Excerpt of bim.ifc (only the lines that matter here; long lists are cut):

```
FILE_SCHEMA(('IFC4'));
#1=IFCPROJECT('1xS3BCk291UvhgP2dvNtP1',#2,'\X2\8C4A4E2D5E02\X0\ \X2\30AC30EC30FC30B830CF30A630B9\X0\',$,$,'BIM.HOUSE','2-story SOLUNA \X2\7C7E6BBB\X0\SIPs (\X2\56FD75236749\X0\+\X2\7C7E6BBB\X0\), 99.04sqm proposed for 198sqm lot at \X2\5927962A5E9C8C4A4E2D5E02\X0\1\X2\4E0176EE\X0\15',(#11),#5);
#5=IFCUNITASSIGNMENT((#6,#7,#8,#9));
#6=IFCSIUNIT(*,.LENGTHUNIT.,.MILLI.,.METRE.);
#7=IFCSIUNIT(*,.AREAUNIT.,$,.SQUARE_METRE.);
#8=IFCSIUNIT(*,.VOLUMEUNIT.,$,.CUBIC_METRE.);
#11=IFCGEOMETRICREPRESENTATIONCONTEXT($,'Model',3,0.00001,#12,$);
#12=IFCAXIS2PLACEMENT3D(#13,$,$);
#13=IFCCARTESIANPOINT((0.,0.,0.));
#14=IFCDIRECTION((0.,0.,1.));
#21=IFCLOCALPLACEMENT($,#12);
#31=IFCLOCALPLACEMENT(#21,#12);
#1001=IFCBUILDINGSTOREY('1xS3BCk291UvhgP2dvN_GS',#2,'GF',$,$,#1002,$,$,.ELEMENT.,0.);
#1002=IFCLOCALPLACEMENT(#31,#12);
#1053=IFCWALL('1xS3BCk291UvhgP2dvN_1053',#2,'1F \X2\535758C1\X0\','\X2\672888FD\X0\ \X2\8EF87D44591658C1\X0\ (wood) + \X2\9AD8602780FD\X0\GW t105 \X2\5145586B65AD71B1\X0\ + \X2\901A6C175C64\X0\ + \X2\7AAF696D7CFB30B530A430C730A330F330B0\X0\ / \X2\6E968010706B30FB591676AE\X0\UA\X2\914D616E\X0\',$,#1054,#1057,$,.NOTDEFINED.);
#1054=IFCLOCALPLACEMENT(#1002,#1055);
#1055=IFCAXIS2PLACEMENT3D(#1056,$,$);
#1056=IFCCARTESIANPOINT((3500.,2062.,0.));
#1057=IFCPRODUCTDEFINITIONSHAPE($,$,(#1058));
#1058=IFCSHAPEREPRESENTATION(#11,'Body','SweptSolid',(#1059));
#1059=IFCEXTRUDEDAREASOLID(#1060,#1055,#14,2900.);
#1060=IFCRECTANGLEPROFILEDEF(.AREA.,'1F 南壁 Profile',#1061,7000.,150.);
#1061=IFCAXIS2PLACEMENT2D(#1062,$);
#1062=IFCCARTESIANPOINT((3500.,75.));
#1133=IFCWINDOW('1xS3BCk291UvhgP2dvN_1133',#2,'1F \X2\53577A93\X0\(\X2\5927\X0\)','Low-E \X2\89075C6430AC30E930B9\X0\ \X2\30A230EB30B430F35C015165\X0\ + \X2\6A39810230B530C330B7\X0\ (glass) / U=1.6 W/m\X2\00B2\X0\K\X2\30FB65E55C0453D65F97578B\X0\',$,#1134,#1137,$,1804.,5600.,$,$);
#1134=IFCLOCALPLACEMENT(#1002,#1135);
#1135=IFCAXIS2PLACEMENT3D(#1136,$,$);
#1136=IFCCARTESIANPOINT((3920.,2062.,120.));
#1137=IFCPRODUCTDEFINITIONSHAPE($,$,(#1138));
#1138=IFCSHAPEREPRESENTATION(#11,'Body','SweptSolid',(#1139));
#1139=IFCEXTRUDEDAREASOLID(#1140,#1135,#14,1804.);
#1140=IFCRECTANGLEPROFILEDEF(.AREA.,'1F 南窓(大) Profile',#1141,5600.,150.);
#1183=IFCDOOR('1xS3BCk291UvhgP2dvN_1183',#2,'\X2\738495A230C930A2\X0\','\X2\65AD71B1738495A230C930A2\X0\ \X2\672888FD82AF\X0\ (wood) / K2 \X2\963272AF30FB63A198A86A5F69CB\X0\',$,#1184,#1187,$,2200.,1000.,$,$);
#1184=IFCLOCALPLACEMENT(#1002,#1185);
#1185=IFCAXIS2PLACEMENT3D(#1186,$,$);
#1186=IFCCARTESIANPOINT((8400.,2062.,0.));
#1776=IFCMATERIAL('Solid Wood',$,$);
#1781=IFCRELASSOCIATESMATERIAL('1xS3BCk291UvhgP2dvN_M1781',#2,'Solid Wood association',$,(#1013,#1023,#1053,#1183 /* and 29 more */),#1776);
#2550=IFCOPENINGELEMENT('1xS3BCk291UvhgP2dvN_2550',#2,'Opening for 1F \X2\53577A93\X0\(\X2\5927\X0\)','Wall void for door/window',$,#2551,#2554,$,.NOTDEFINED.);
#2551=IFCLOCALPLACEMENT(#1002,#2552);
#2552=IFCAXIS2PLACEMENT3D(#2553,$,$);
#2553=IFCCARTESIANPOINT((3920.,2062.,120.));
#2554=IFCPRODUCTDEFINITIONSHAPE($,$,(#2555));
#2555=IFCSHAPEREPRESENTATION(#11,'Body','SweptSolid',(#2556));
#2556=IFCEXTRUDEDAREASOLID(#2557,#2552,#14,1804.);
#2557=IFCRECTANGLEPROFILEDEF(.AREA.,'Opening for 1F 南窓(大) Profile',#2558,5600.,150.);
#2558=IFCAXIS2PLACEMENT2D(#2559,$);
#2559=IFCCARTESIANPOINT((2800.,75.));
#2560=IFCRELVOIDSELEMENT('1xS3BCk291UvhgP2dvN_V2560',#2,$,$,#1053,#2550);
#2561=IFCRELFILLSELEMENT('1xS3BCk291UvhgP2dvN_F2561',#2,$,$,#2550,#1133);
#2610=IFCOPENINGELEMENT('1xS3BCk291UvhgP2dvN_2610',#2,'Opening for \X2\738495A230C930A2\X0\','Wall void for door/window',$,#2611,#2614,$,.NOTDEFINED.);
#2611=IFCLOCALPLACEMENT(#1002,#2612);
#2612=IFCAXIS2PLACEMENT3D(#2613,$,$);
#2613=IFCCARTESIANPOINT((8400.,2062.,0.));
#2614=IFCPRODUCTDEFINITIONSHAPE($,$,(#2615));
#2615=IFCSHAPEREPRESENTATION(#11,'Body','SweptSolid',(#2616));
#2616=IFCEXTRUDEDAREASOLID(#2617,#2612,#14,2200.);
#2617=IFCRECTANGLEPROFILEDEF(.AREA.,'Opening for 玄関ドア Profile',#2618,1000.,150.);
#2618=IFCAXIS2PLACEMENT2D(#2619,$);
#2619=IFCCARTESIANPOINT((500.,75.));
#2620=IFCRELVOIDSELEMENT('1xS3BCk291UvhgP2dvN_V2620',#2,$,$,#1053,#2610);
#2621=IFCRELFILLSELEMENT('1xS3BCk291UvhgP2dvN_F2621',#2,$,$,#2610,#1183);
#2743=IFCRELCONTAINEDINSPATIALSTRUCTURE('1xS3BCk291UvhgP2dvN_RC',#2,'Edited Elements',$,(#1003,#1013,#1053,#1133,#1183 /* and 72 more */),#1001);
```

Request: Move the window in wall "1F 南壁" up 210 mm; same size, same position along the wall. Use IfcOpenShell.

```python
import numpy as np
import ifcopenshell
import ifcopenshell.api.geometry
import ifcopenshell.util.placement
import ifcopenshell.util.unit

model = ifcopenshell.open("bim.ifc")
unit_scale = ifcopenshell.util.unit.calculate_unit_scale(model)

window = model.by_guid("1xS3BCk291UvhgP2dvN_1133")
opening = window.FillsVoids[0].RelatingOpeningElement
dz = 0.21 / unit_scale

shift = np.array([0.0, 0.0, dz])
# The window is not placed relative to its opening, so move both.
for product in (opening, window):
    matrix = ifcopenshell.util.placement.get_local_placement(product.ObjectPlacement)
    matrix[:3, 3] += shift
    ifcopenshell.api.geometry.edit_object_placement(model, product=product, matrix=matrix, is_si=False)

print(f"moved by {dz * unit_scale:+.3f} m")

model.write("bim_updated.ifc")
```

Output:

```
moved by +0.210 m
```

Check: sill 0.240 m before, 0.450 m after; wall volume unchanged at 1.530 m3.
